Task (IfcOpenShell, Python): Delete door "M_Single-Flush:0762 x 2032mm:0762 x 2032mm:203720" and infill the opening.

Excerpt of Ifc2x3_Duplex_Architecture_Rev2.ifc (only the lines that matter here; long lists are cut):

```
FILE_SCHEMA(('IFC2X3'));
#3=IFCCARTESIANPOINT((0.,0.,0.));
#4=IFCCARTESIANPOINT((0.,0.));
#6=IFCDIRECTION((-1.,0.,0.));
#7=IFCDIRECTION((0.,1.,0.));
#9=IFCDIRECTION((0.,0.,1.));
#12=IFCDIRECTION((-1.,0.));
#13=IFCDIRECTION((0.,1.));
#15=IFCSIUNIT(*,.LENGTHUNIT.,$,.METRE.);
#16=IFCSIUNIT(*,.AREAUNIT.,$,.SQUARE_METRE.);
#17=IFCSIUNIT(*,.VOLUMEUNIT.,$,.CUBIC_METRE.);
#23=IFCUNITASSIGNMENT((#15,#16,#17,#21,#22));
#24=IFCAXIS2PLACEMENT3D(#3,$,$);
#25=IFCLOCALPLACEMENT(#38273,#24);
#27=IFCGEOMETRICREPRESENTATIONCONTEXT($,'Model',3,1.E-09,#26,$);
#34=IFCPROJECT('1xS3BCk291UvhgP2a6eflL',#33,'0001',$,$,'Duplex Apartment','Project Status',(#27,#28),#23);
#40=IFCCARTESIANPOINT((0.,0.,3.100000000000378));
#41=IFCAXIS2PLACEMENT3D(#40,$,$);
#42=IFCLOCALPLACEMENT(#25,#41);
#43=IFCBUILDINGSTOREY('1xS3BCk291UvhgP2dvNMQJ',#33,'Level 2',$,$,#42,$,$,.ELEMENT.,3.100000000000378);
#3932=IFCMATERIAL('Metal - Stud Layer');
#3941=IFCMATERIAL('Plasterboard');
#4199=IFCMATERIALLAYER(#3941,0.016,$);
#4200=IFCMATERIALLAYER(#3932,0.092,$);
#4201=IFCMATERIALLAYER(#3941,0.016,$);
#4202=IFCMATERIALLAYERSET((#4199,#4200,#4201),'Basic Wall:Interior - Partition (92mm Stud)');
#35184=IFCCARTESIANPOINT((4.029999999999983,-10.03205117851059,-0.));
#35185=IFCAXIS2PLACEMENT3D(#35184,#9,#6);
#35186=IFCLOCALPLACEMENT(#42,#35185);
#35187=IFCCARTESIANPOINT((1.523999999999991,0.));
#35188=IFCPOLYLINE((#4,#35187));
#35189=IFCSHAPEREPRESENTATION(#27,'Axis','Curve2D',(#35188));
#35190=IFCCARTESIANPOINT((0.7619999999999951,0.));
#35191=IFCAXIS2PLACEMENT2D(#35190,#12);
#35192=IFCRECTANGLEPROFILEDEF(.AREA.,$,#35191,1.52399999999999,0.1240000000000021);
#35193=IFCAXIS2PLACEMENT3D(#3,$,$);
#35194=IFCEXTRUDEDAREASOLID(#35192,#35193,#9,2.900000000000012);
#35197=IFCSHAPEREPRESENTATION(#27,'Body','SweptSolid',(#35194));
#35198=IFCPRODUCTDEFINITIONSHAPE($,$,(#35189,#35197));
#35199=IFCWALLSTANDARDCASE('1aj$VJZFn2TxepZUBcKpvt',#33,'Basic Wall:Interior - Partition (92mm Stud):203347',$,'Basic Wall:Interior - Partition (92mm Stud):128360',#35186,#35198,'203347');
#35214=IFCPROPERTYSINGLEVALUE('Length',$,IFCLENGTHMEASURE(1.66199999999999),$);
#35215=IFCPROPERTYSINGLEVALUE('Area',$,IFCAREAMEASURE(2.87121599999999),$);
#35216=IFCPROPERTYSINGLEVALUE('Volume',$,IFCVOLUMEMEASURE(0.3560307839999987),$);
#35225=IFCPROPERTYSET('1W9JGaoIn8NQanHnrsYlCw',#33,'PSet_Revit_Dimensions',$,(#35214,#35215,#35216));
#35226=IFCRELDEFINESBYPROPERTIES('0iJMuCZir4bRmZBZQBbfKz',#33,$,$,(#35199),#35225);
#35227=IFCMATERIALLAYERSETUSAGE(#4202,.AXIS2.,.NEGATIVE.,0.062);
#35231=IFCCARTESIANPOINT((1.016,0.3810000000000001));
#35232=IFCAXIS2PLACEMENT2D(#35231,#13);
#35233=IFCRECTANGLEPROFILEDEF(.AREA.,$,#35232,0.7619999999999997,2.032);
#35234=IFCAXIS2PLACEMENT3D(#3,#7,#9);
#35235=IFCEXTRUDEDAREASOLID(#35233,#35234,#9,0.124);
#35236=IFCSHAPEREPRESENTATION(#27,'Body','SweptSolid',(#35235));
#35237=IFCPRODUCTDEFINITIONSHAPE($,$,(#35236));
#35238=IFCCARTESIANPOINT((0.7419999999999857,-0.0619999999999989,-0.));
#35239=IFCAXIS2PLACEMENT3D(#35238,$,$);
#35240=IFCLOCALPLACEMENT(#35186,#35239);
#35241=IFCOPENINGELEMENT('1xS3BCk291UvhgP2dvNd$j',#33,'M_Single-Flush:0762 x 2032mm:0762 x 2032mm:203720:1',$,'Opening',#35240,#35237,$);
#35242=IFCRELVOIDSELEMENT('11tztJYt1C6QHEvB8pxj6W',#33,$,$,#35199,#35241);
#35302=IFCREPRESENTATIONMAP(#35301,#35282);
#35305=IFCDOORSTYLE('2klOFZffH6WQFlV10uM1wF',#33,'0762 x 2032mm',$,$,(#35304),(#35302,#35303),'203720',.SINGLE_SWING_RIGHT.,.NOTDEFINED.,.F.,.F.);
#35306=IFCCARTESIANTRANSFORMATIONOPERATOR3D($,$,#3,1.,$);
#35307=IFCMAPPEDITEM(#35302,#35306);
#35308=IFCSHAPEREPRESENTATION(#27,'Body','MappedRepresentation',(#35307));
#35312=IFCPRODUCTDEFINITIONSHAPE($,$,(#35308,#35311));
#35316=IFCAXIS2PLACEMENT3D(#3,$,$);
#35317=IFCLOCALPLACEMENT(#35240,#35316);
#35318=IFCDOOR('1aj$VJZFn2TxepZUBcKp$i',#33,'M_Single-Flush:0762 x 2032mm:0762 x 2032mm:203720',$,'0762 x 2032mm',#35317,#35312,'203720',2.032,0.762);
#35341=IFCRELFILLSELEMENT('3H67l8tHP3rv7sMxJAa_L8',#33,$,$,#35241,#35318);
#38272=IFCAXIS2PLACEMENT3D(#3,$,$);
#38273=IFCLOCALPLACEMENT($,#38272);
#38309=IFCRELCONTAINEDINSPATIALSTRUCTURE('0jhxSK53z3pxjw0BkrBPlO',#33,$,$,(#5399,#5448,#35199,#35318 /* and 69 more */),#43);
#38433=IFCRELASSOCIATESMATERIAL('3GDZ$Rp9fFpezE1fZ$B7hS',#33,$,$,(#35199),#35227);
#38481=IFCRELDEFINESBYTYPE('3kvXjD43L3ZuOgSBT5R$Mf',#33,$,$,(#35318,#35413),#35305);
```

```python
import ifcopenshell
import ifcopenshell.api.feature
import ifcopenshell.api.pset
import ifcopenshell.api.root
import ifcopenshell.geom
import ifcopenshell.util.element
import ifcopenshell.util.shape
import ifcopenshell.util.unit

model = ifcopenshell.open("Ifc2x3_Duplex_Architecture_Rev2.ifc")
area_scale = ifcopenshell.util.unit.calculate_unit_scale(model, "AREAUNIT")
volume_scale = ifcopenshell.util.unit.calculate_unit_scale(model, "VOLUMEUNIT")
settings = ifcopenshell.geom.settings()


def volume(element):
    """Net volume in cubic metres, openings subtracted."""
    shape = ifcopenshell.geom.create_shape(settings, element)
    return ifcopenshell.util.shape.get_volume(shape.geometry)


door = model.by_id(35318)
opening = door.FillsVoids[0].RelatingOpeningElement
wall = opening.VoidsElements[0].RelatingBuildingElement
before = volume(wall)

ifcopenshell.api.root.remove_product(model, product=door)
ifcopenshell.api.feature.remove_feature(model, feature=opening)

after = volume(wall)
thickness = 0.124  # wall thickness in metres

# Update the wall's stored quantities.
pset = model.by_id(ifcopenshell.util.element.get_pset(wall, "PSet_Revit_Dimensions", should_inherit=False)["id"])
ifcopenshell.api.pset.edit_pset(model, pset=pset, properties={
    "Area": model.create_entity("IfcAreaMeasure", after / thickness / area_scale),
    "Volume": model.create_entity("IfcVolumeMeasure", after / volume_scale),
})

print(f"wall volume {before:.3f} -> {after:.3f} m3")

model.write("Ifc2x3_Duplex_Architecture_Rev2-out.ifc")
```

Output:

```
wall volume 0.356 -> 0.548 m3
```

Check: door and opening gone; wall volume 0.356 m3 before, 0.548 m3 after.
